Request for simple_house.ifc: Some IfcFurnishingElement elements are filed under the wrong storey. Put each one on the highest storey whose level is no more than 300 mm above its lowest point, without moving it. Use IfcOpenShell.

First a look at what the model holds.

```python
import ifcopenshell
import ifcopenshell.util.element
import ifcopenshell.util.placement

model = ifcopenshell.open("simple_house.ifc")
print(model.schema)
for storey in model.by_type("IfcBuildingStorey"):
    level = ifcopenshell.util.placement.get_storey_elevation(storey)
    count = sum(e.is_a("IfcFurnishingElement") for e in ifcopenshell.util.element.get_contained(storey))
    print(storey.id(), storey.Name, round(level, 3), count, sep=" | ")
```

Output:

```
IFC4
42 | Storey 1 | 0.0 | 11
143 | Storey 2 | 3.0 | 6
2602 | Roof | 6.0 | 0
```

```python
import ifcopenshell
import ifcopenshell.api.spatial
import ifcopenshell.geom
import ifcopenshell.util.element
import ifcopenshell.util.placement
import ifcopenshell.util.shape
import ifcopenshell.util.unit

model = ifcopenshell.open("simple_house.ifc")
unit_scale = ifcopenshell.util.unit.calculate_unit_scale(model)
settings = ifcopenshell.geom.settings()

levels = sorted(
    ((ifcopenshell.util.placement.get_storey_elevation(s) * unit_scale, s) for s in model.by_type("IfcBuildingStorey")),
    key=lambda pair: pair[0],
)

for e in model.by_type("IfcFurnishingElement"):
    current = e.ContainedInStructure[0].RelatingStructure if e.ContainedInStructure else None
    if current is None or not current.is_a("IfcBuildingStorey"):
        continue
    shape = ifcopenshell.geom.create_shape(settings, e)
    bottom = ifcopenshell.util.shape.get_shape_bottom_elevation(shape, shape.geometry)
    below = [s for level, s in levels if level <= bottom + 0.3]
    storey = below[-1] if below else levels[0][1]
    if storey != current:
        # assign_container keeps the world position.
        ifcopenshell.api.spatial.assign_container(model, products=[e], relating_structure=storey)
        print(e.id(), current.Name, "->", storey.Name)

model.write("simple_house-out.ifc")
```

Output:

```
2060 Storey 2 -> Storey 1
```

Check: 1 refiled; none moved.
